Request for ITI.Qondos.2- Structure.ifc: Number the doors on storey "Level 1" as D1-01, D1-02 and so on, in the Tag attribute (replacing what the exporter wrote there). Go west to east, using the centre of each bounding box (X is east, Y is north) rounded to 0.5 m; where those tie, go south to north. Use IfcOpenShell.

First a look at what the model holds.

```python
import ifcopenshell
import ifcopenshell.util.element
import ifcopenshell.util.placement

model = ifcopenshell.open("ITI.Qondos.2- Structure.ifc")
print(model.schema)
storey = next(s for s in model.by_type("IfcBuildingStorey") if s.Name == "Level 1")
doors = [e for e in ifcopenshell.util.element.get_decomposition(storey) if e.is_a("IfcDoor")]
for e in sorted(doors, key=lambda e: e.id()):
    origin = ifcopenshell.util.placement.get_local_placement(e.ObjectPlacement)[:3, 3]
    print(e.id(), e.Tag, e.Name, origin.round(2) + 0.0, sep=" | ")
```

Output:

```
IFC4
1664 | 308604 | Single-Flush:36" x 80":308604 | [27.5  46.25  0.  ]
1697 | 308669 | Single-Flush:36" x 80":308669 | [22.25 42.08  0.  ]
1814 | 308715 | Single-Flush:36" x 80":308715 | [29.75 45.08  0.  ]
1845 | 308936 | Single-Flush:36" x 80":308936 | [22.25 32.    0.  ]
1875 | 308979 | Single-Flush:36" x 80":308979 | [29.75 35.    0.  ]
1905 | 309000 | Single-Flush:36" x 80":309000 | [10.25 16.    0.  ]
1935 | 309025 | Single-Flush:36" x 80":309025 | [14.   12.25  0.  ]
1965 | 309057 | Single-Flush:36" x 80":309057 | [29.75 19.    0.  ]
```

```python
import ifcopenshell
import ifcopenshell.geom
import ifcopenshell.util.element
import ifcopenshell.util.shape

model = ifcopenshell.open("ITI.Qondos.2- Structure.ifc")
settings = ifcopenshell.geom.settings()
settings.set("use-world-coords", True)


def centre(element):
    shape = ifcopenshell.geom.create_shape(settings, element)
    return ifcopenshell.util.shape.get_bbox_centroid(shape.geometry)


storey = next(s for s in model.by_type("IfcBuildingStorey") if s.Name == "Level 1")
doors = [e for e in ifcopenshell.util.element.get_decomposition(storey) if e.is_a("IfcDoor")]

# Insertion points can sit at a corner or the storey origin, so sort by the geometry (in metres).
centres = {e: centre(e) for e in doors}
doors.sort(key=lambda e: (round(centres[e][0] / 0.5), centres[e][1]))

for i, e in enumerate(doors, start=1):
    number = f"D1-{i:02d}"
    e.Tag = number
    print(e.id(), number)

model.write("ITI.Qondos.2- Structure_rev.ifc")
```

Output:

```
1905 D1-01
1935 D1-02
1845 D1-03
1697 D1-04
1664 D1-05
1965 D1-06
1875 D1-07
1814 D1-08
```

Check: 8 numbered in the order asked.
